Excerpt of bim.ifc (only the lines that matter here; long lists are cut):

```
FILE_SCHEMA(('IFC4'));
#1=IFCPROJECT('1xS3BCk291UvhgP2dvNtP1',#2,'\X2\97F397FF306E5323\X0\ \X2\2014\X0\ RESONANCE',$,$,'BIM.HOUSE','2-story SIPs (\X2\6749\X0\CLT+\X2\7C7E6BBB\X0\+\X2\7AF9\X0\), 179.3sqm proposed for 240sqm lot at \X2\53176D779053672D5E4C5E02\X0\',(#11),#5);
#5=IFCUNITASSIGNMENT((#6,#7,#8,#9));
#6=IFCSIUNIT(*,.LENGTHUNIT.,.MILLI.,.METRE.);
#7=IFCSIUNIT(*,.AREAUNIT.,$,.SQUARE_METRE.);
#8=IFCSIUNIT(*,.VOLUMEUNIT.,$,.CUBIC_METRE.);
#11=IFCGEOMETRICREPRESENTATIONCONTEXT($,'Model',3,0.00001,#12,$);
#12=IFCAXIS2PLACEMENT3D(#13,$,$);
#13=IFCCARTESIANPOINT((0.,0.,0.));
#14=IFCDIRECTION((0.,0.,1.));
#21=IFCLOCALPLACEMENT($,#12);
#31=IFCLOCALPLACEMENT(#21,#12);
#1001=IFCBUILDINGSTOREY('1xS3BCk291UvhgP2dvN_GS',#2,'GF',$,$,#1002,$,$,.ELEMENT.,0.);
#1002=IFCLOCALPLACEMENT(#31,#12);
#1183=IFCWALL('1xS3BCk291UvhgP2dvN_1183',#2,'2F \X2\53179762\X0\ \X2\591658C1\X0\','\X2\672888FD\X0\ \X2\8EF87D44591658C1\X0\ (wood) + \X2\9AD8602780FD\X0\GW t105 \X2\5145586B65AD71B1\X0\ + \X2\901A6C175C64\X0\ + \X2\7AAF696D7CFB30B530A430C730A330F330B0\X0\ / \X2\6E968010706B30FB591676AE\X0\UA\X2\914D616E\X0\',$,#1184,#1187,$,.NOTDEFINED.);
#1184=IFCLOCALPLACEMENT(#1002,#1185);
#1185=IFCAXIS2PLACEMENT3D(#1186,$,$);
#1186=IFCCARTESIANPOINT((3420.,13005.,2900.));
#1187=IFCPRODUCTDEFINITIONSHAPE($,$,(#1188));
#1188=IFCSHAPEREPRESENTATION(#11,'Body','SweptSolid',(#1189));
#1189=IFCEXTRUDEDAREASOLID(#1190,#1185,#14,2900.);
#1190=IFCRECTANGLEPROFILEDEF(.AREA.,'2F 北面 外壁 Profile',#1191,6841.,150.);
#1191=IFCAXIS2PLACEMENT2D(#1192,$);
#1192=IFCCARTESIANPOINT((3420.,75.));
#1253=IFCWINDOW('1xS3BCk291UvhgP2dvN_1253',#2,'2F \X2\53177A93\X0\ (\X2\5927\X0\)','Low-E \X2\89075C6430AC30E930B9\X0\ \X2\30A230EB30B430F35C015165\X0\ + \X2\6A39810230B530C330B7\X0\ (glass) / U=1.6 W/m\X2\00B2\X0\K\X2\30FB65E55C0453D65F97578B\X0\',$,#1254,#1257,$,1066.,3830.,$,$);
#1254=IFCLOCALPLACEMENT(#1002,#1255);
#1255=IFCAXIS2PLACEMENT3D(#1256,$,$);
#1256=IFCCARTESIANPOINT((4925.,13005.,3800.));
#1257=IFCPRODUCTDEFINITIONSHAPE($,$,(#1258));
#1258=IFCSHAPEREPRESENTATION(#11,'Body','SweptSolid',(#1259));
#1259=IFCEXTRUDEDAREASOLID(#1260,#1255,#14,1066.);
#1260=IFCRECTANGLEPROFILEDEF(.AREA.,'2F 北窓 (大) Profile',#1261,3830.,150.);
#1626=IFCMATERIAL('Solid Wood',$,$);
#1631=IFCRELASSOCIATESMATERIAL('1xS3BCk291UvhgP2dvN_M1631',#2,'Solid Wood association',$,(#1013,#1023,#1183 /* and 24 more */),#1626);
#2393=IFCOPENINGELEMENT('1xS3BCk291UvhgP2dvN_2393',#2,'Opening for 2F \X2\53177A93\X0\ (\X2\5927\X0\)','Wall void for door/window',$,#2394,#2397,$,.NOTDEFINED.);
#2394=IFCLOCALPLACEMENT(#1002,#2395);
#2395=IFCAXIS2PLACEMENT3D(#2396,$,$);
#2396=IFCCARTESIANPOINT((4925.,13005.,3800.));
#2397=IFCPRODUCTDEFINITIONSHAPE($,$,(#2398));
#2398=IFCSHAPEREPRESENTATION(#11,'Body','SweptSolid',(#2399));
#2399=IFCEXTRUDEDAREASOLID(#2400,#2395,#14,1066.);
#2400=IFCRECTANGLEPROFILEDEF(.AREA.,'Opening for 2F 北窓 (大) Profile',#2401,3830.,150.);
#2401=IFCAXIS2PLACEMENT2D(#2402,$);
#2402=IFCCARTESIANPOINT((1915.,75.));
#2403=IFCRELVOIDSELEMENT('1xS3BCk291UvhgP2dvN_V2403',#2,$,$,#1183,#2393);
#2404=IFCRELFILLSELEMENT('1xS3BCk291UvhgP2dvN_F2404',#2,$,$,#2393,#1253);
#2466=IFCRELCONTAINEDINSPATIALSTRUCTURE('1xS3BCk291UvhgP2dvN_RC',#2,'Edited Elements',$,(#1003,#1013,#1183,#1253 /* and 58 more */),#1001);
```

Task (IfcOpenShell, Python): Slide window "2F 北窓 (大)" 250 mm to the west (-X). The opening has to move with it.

```python
import ifcopenshell
import ifcopenshell.api.geometry
import ifcopenshell.util.placement
import ifcopenshell.util.unit

model = ifcopenshell.open("bim.ifc")
unit_scale = ifcopenshell.util.unit.calculate_unit_scale(model)

window = model.by_guid("1xS3BCk291UvhgP2dvN_1253")
opening = window.FillsVoids[0].RelatingOpeningElement
wall = opening.VoidsElements[0].RelatingBuildingElement

wall_matrix = ifcopenshell.util.placement.get_local_placement(wall.ObjectPlacement)
shift = wall_matrix[:3, 0] * -0.25 / unit_scale
before = ifcopenshell.util.placement.get_local_placement(window.ObjectPlacement)[:3, 3].copy()

# The window is not placed relative to its opening, so move both.
for product in (opening, window):
    matrix = ifcopenshell.util.placement.get_local_placement(product.ObjectPlacement)
    matrix[:3, 3] += shift
    ifcopenshell.api.geometry.edit_object_placement(model, product=product, matrix=matrix, is_si=False)

after = ifcopenshell.util.placement.get_local_placement(window.ObjectPlacement)[:3, 3]
print("window moved by", (after - before).round(3) + 0.0)

model.write("bim_updated.ifc")
```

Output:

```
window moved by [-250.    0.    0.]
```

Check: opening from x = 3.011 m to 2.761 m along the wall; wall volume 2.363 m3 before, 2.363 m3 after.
